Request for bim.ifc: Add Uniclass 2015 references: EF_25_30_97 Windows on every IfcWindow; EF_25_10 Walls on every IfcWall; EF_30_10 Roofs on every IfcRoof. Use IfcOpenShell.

First a look at what the model holds.

```python
import ifcopenshell

model = ifcopenshell.open("bim.ifc")
print(model.schema)
print("classifications:", [c.Name for c in model.by_type("IfcClassification")])
for ifc_class in ("IfcDoor", "IfcRoof", "IfcStair", "IfcWall", "IfcWindow"):
    print(ifc_class, len(model.by_type(ifc_class)))
```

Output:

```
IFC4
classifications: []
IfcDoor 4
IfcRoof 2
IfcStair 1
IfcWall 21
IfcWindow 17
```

```python
import ifcopenshell
import ifcopenshell.api.classification

model = ifcopenshell.open("bim.ifc")

system = ifcopenshell.api.classification.add_classification(model, classification="Uniclass 2015")

codes = {
    "IfcWindow": ("EF_25_30_97", "Windows"),
    "IfcWall": ("EF_25_10", "Walls"),
    "IfcRoof": ("EF_30_10", "Roofs"),
}
for ifc_class, (code, name) in codes.items():
    products = model.by_type(ifc_class)
    ifcopenshell.api.classification.add_reference(
        model, products=products, classification=system, identification=code, name=name
    )
    print(code, len(products))

model.write("bim_rev.ifc")
```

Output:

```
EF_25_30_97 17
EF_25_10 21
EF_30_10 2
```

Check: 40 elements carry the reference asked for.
